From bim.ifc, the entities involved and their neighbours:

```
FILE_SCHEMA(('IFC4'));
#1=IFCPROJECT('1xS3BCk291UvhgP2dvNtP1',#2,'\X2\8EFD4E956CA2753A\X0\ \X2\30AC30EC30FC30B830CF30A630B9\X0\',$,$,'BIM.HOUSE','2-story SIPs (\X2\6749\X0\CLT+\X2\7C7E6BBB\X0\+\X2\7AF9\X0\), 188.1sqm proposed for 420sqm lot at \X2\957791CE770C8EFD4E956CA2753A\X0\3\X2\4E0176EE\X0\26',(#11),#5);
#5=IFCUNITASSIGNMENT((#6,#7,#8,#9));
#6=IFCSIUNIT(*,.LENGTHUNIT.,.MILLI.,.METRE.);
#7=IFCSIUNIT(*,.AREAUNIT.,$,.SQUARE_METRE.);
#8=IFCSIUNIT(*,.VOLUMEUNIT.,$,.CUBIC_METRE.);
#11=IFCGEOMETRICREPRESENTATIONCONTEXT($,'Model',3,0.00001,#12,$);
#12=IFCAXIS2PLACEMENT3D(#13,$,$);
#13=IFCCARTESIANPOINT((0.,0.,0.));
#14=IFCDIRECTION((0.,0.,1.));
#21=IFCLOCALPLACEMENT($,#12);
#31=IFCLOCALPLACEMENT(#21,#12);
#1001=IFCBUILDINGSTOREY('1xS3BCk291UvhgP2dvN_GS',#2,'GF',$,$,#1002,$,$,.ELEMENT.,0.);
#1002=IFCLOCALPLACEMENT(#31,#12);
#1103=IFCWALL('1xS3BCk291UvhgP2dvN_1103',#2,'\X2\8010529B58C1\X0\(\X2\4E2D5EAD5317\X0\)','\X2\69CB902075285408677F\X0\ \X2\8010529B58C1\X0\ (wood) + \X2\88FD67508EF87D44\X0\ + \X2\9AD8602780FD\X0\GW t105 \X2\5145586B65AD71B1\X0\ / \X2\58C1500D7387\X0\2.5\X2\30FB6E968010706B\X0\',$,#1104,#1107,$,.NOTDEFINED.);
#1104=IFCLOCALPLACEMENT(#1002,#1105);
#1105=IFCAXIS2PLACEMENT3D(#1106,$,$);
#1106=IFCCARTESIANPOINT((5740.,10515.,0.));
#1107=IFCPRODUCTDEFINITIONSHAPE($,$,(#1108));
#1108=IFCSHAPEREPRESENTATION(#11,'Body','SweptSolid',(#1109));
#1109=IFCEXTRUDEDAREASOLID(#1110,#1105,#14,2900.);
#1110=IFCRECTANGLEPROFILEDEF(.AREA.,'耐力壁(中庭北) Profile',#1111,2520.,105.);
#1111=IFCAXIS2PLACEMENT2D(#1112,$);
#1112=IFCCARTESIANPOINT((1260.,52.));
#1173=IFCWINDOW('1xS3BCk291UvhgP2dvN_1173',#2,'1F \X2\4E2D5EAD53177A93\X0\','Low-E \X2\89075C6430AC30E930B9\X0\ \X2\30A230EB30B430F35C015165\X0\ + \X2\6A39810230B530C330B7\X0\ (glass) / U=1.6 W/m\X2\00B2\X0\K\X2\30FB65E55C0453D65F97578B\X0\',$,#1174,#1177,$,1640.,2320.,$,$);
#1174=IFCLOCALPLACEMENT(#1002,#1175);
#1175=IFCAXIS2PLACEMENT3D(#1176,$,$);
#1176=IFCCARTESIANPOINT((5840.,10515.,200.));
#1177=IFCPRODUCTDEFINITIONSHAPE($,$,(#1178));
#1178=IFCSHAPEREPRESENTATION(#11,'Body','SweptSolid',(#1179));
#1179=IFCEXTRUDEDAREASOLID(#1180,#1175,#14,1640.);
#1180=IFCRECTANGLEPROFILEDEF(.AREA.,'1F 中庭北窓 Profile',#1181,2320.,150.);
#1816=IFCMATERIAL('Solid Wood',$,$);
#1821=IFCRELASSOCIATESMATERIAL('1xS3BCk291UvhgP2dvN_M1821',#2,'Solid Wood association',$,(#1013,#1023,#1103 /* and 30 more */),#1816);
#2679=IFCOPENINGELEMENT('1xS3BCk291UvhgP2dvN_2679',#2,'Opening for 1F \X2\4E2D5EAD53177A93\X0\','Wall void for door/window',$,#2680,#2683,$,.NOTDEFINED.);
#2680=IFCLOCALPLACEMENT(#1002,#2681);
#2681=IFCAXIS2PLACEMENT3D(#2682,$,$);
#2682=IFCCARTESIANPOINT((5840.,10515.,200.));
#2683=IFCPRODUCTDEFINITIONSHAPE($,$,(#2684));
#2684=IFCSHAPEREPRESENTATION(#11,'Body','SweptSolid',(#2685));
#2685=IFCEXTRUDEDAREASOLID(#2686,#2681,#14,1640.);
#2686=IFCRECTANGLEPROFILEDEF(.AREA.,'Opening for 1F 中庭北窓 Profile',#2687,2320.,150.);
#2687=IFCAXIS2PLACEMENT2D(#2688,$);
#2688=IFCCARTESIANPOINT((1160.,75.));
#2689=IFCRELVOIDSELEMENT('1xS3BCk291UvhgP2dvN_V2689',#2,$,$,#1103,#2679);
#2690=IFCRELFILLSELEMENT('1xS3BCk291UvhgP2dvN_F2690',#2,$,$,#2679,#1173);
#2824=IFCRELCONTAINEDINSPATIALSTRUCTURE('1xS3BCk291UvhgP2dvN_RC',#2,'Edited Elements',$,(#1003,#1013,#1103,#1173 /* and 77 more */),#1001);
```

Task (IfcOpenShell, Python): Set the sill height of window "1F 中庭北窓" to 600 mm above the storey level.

```python
import numpy as np
import ifcopenshell
import ifcopenshell.api.geometry
import ifcopenshell.geom
import ifcopenshell.util.element
import ifcopenshell.util.placement
import ifcopenshell.util.shape
import ifcopenshell.util.unit

model = ifcopenshell.open("bim.ifc")
unit_scale = ifcopenshell.util.unit.calculate_unit_scale(model)

window = model.by_guid("1xS3BCk291UvhgP2dvN_1173")
opening = window.FillsVoids[0].RelatingOpeningElement
storey = ifcopenshell.util.element.get_container(window, ifc_class="IfcBuildingStorey")
level = ifcopenshell.util.placement.get_local_placement(storey.ObjectPlacement)[2, 3]

# The opening's origin need not be at the sill, so measure its lowest point.
shape = ifcopenshell.geom.create_shape(ifcopenshell.geom.settings(), opening)
bottom = ifcopenshell.util.shape.get_shape_bottom_elevation(shape, shape.geometry) / unit_scale
dz = level + 0.6 / unit_scale - bottom

shift = np.array([0.0, 0.0, dz])
# The window is not placed relative to its opening, so move both.
for product in (opening, window):
    matrix = ifcopenshell.util.placement.get_local_placement(product.ObjectPlacement)
    matrix[:3, 3] += shift
    ifcopenshell.api.geometry.edit_object_placement(model, product=product, matrix=matrix, is_si=False)

print(f"moved by {dz * unit_scale:+.3f} m")

model.write("bim_updated.ifc")
```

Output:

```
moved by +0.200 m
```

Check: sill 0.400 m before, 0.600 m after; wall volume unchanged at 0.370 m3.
